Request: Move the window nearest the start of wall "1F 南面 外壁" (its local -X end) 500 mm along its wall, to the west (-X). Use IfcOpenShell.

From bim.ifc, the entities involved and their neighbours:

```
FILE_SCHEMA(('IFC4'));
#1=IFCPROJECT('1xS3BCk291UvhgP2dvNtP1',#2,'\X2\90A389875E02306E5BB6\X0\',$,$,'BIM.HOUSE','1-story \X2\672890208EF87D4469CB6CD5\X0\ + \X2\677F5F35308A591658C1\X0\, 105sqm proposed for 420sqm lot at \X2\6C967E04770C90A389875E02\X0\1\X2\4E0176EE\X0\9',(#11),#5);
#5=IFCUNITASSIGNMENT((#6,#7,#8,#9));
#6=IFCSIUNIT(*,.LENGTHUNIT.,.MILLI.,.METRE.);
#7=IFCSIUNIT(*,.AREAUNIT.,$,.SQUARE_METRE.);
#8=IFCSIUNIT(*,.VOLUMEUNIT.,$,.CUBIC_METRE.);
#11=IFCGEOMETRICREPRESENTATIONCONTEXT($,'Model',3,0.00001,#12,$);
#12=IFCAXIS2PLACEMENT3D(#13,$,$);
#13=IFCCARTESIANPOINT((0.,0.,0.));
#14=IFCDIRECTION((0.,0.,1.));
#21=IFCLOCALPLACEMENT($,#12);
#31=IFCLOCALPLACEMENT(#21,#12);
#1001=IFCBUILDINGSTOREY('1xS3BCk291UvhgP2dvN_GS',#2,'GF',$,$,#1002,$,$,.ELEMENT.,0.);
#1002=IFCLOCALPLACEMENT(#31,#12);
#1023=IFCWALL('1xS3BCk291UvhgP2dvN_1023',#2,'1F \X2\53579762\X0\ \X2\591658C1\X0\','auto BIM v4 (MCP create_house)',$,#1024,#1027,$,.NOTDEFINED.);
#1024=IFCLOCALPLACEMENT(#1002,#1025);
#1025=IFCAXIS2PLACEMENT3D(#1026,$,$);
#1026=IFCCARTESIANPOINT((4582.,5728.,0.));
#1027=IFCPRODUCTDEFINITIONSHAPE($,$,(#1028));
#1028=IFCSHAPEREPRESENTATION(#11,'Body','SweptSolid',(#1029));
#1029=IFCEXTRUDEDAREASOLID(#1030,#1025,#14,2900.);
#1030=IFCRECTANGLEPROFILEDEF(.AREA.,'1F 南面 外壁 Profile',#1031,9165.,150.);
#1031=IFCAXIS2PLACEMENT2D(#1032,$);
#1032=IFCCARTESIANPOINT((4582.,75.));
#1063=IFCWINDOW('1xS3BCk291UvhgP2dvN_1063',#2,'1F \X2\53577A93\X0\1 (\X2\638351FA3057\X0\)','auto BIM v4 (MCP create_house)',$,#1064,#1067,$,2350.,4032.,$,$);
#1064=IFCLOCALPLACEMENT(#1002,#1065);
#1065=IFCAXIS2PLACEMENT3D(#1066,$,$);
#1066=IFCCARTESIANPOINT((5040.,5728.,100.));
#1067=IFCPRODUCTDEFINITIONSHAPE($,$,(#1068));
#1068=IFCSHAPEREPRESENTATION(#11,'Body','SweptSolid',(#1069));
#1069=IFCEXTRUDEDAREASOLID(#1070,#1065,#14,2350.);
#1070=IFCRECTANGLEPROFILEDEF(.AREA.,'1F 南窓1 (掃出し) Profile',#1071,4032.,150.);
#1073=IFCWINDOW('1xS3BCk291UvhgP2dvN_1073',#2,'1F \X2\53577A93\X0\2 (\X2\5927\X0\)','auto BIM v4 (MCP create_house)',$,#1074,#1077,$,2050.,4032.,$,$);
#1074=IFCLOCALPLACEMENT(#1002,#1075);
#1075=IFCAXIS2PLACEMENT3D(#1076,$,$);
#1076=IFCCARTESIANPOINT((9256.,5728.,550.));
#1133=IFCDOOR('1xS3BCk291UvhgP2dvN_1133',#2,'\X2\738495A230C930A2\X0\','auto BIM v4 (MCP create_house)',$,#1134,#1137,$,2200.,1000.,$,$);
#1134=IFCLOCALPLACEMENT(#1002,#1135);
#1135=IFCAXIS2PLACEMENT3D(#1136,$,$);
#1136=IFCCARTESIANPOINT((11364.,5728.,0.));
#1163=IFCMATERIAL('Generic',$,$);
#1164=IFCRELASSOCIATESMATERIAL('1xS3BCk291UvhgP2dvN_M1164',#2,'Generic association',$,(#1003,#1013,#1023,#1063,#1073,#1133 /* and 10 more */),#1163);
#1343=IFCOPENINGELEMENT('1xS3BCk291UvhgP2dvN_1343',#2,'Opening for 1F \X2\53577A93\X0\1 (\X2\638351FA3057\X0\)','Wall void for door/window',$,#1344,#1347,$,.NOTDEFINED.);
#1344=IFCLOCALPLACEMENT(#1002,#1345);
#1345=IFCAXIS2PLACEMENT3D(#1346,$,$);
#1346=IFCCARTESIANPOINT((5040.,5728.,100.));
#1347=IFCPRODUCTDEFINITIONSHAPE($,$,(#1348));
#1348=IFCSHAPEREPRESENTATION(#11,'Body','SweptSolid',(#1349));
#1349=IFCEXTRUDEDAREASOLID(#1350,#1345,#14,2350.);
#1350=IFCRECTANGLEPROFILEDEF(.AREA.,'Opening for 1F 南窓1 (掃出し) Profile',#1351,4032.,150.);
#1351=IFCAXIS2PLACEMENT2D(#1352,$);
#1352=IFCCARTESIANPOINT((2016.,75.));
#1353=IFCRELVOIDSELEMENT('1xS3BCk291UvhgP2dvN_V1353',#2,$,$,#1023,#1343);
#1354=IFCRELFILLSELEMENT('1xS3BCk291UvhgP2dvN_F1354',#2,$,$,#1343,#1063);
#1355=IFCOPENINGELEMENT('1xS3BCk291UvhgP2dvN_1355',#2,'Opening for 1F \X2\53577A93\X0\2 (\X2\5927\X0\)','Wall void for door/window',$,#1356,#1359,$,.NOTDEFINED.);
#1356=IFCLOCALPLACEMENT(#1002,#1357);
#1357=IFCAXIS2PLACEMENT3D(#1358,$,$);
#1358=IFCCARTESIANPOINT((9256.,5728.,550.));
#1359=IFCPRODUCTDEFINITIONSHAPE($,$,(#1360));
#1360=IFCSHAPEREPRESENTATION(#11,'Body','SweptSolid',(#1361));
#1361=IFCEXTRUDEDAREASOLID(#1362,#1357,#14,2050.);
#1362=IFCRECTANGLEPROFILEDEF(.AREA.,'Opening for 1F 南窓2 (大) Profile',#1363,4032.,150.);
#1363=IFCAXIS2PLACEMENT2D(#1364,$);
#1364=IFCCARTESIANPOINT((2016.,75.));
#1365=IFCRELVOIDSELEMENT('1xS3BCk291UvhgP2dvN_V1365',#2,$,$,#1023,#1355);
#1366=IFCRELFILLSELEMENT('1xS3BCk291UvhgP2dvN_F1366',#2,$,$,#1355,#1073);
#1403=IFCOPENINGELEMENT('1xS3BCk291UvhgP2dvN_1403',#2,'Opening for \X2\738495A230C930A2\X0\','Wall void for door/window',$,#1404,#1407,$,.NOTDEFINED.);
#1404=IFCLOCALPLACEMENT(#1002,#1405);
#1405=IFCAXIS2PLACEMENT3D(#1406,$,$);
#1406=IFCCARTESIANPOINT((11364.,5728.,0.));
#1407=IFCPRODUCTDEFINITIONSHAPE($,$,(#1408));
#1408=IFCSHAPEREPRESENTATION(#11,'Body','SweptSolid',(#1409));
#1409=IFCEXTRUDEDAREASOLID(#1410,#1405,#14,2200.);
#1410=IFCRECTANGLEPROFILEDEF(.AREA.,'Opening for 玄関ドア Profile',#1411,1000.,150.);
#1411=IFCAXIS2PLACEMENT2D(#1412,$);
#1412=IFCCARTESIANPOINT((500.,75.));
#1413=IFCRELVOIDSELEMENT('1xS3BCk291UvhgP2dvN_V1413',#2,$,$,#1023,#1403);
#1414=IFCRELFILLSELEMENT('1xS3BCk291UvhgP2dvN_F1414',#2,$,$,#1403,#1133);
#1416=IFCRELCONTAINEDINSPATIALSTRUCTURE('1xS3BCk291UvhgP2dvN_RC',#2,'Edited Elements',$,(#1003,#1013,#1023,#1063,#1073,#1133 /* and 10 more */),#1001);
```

```python
import ifcopenshell
import ifcopenshell.api.geometry
import ifcopenshell.util.placement

model = ifcopenshell.open("bim.ifc")

window = model.by_guid("1xS3BCk291UvhgP2dvN_1063")
opening = window.FillsVoids[0].RelatingOpeningElement
wall = opening.VoidsElements[0].RelatingBuildingElement

wall_matrix = ifcopenshell.util.placement.get_local_placement(wall.ObjectPlacement)
shift = wall_matrix[:3, 0] * -500.0
before = ifcopenshell.util.placement.get_local_placement(window.ObjectPlacement)[:3, 3].copy()

# The window is not placed relative to its opening, so move both.
for product in (opening, window):
    matrix = ifcopenshell.util.placement.get_local_placement(product.ObjectPlacement)
    matrix[:3, 3] += shift
    ifcopenshell.api.geometry.edit_object_placement(model, product=product, matrix=matrix, is_si=False)

after = ifcopenshell.util.placement.get_local_placement(window.ObjectPlacement)[:3, 3]
print("window moved by", (after - before).round(3) + 0.0)

model.write("bim_updated.ifc")
```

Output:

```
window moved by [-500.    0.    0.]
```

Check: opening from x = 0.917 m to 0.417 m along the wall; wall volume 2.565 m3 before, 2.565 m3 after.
